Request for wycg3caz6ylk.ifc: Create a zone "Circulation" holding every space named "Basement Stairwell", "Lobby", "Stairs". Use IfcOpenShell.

First a look at what the model holds.

```python
import ifcopenshell

model = ifcopenshell.open("wycg3caz6ylk.ifc")
print(model.schema)
seen = {}
for space in model.by_type("IfcSpace"):
    seen[space.Name] = seen.get(space.Name, 0) + 1
for name, count in sorted(seen.items(), key=str):
    print(count, "x", name)
print("zones:", [z.Name for z in model.by_type("IfcZone")][:20])
```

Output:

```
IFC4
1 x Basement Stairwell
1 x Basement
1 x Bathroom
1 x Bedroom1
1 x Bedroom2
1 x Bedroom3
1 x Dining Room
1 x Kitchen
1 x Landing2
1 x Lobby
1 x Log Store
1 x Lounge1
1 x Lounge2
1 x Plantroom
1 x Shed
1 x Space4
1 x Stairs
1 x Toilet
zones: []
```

```python
import ifcopenshell
import ifcopenshell.api.group
import ifcopenshell.api.root

model = ifcopenshell.open("wycg3caz6ylk.ifc")

names = {"Basement Stairwell", "Lobby", "Stairs"}
spaces = [s for s in model.by_type("IfcSpace") if s.Name in names]

zone = ifcopenshell.api.root.create_entity(model, ifc_class="IfcZone", name="Circulation")
ifcopenshell.api.group.assign_group(model, products=spaces, group=zone)
print(len(spaces), "spaces in", zone.Name)

model.write("wycg3caz6ylk_updated.ifc")
```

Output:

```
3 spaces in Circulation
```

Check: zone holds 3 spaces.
